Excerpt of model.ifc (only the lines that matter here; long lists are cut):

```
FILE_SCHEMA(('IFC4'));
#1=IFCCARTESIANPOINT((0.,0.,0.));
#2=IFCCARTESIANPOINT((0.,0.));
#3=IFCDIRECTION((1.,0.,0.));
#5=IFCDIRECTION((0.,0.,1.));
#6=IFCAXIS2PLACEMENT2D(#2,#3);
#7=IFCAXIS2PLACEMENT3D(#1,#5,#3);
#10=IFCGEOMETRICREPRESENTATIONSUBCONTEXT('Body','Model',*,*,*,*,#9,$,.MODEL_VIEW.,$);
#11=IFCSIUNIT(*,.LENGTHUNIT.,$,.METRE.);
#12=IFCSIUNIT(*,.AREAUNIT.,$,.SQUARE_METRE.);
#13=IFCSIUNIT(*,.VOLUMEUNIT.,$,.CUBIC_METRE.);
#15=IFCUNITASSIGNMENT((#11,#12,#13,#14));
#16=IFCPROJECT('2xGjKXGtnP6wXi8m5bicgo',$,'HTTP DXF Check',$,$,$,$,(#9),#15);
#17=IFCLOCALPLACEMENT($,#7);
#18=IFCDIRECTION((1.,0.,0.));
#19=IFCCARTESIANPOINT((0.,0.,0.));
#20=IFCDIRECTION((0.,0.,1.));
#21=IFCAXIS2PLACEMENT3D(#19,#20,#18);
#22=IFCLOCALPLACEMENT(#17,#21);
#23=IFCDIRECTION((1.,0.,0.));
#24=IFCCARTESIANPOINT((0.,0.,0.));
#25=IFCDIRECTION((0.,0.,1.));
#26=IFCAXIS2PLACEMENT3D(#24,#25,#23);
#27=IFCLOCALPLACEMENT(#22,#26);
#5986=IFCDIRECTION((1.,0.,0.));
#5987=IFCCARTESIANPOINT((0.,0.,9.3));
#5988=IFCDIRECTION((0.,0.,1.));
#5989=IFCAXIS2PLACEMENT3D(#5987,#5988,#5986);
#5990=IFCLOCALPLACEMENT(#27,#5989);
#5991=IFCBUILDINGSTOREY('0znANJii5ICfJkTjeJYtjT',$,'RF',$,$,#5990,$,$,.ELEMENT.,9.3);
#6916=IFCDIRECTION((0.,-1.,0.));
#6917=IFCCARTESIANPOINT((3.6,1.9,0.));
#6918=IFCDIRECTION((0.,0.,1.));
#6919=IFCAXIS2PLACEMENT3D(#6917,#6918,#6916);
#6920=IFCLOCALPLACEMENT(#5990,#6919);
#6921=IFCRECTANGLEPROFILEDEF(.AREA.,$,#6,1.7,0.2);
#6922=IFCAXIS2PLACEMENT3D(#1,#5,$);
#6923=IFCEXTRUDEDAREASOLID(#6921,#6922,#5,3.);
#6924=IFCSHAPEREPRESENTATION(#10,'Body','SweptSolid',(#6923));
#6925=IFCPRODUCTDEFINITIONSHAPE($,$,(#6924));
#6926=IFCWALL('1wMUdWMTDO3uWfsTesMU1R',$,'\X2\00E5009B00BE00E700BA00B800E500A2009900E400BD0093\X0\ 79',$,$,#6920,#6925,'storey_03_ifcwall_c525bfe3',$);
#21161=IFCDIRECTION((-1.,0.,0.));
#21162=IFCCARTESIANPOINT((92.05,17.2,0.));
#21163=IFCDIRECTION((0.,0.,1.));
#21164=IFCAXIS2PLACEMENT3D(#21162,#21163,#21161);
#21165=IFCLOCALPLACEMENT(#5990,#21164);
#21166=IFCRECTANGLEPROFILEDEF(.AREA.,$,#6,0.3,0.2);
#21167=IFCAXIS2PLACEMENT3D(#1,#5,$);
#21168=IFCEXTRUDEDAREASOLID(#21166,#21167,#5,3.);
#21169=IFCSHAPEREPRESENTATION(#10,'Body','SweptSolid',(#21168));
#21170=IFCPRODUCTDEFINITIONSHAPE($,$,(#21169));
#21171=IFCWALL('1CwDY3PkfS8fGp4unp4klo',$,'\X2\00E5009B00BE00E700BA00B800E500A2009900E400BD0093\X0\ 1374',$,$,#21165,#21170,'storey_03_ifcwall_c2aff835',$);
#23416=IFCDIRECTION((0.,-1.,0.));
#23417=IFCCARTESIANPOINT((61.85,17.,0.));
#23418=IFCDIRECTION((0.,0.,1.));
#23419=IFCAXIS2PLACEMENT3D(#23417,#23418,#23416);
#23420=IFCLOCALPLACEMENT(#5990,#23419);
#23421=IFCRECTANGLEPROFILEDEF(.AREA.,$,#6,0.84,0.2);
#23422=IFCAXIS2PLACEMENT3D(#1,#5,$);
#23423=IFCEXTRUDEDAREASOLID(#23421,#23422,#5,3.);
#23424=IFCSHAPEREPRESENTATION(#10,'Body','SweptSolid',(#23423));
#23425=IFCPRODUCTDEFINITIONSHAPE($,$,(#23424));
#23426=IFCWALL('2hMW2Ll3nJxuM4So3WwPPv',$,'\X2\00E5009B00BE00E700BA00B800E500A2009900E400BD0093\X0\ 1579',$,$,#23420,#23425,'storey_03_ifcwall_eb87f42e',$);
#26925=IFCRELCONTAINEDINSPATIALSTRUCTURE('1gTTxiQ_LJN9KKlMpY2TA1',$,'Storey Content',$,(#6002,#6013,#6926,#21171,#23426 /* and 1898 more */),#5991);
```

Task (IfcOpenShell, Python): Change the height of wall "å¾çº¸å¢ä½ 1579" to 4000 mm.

```python
import ifcopenshell
import ifcopenshell.geom
import ifcopenshell.util.representation
import ifcopenshell.util.shape
import ifcopenshell.util.unit

model = ifcopenshell.open("model.ifc")
unit_scale = ifcopenshell.util.unit.calculate_unit_scale(model)
settings = ifcopenshell.geom.settings()


def volume(element):
    """Net volume in cubic metres, openings subtracted."""
    shape = ifcopenshell.geom.create_shape(settings, element)
    return ifcopenshell.util.shape.get_volume(shape.geometry)


wall = model.by_guid("2hMW2Ll3nJxuM4So3WwPPv")
before = volume(wall)

body = ifcopenshell.util.representation.get_representation(wall, "Model", "Body")
solid = body.Items[0]
old_height = solid.Depth
solid.Depth = 4 / unit_scale
after = volume(wall)

print(f"height {old_height:g} -> {solid.Depth:g}, volume {before:.3f} -> {after:.3f} m3")

model.write("model-out.ifc")
```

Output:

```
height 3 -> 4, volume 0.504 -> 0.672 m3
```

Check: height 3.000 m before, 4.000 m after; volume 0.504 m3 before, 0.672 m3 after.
